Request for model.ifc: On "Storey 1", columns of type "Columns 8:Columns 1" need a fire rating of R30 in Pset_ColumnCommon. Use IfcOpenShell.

First a look at what the model holds.

```python
import ifcopenshell
import ifcopenshell.util.element

model = ifcopenshell.open("model.ifc")
print(model.schema)
storey = next(s for s in model.by_type("IfcBuildingStorey") if s.Name == "Storey 1")
columns = [e for e in ifcopenshell.util.element.get_decomposition(storey) if e.is_a("IfcColumn")]
seen = {}
for e in columns:
    element_type = ifcopenshell.util.element.get_type(e)
    key = (element_type.Name if element_type != e and element_type else None, ifcopenshell.util.element.get_pset(e, "Pset_ColumnCommon", "FireRating"))
    seen[key] = seen.get(key, 0) + 1
for (name, value), count in sorted(seen.items(), key=str):
    print(count, "x", name, "|", value)
```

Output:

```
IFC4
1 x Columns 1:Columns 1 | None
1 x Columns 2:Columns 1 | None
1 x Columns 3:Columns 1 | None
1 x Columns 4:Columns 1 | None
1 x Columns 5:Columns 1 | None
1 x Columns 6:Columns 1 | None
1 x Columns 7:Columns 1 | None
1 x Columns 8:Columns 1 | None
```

```python
import ifcopenshell
import ifcopenshell.api.pset
import ifcopenshell.util.element

model = ifcopenshell.open("model.ifc")

storey = next(s for s in model.by_type("IfcBuildingStorey") if s.Name == "Storey 1")
columns = [e for e in ifcopenshell.util.element.get_decomposition(storey) if e.is_a("IfcColumn")]

count = 0
for e in columns:
    element_type = ifcopenshell.util.element.get_type(e)
    if element_type in (None, e) or element_type.Name != "Columns 8:Columns 1":
        continue
    # add_pset returns the element's existing set when there is one.
    pset = ifcopenshell.api.pset.add_pset(model, product=e, name="Pset_ColumnCommon")
    ifcopenshell.api.pset.edit_pset(model, pset=pset, properties={"FireRating": "R30"})
    count += 1

print(count, "columns updated")

model.write("model_updated.ifc")
```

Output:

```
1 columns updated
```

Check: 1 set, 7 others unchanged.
